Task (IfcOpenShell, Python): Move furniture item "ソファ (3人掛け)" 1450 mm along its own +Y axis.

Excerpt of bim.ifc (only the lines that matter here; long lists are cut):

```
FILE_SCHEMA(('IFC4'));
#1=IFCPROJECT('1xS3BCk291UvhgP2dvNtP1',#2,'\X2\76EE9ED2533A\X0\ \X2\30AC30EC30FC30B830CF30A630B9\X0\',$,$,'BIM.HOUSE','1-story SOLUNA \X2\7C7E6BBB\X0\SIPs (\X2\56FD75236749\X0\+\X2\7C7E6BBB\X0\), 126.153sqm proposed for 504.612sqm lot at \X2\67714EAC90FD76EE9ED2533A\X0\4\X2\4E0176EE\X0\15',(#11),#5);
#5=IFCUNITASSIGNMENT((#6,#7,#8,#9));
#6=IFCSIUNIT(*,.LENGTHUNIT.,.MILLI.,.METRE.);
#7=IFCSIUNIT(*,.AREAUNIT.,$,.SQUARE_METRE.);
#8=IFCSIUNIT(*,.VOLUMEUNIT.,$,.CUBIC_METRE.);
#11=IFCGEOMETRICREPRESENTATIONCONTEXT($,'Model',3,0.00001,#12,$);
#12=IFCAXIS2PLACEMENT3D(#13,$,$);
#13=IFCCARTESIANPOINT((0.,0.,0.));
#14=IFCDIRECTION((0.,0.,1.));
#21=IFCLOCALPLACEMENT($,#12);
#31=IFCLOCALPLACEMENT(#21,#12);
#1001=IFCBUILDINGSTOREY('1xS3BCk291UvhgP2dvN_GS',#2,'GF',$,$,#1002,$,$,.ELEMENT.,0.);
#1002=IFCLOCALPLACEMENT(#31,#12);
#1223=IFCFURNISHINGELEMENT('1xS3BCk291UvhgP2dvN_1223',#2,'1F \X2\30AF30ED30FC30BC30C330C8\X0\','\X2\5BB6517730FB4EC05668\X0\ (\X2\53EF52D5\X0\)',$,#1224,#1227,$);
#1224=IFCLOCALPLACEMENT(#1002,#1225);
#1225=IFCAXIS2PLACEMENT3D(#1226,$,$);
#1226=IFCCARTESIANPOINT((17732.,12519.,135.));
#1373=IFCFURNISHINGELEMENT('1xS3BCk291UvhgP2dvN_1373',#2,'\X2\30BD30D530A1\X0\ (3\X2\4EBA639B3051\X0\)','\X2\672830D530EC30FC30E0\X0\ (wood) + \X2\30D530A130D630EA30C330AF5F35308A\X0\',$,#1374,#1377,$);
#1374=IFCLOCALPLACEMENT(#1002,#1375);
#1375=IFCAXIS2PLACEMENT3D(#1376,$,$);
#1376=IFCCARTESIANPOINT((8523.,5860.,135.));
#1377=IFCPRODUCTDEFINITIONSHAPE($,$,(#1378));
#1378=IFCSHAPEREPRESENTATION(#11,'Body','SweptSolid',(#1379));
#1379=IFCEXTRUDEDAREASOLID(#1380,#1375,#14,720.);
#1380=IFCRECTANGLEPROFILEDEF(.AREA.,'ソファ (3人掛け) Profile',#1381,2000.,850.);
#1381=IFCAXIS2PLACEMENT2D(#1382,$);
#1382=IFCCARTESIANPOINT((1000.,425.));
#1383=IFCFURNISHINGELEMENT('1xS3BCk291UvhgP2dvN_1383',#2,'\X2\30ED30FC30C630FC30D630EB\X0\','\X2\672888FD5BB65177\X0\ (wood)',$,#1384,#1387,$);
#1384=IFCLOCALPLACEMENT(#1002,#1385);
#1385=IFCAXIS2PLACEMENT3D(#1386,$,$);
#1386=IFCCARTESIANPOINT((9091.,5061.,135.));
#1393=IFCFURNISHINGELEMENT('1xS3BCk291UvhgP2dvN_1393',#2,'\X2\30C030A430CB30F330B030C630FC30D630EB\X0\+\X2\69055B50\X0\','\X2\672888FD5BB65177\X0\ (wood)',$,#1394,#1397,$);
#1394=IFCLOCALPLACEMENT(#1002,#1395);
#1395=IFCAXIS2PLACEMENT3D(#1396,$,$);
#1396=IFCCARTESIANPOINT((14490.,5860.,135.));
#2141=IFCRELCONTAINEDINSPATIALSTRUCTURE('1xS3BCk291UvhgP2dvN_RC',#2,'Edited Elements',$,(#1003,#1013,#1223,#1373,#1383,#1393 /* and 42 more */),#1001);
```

```python
import ifcopenshell
import ifcopenshell.api.geometry
import ifcopenshell.util.placement
import ifcopenshell.util.unit

model = ifcopenshell.open("bim.ifc")
unit_scale = ifcopenshell.util.unit.calculate_unit_scale(model)

item = model.by_guid("1xS3BCk291UvhgP2dvN_1373")
matrix = ifcopenshell.util.placement.get_local_placement(item.ObjectPlacement)
matrix[:3, 3] += matrix[:3, 1] * 1.45 / unit_scale
ifcopenshell.api.geometry.edit_object_placement(model, product=item, matrix=matrix, is_si=False)

print(ifcopenshell.util.placement.get_local_placement(item.ObjectPlacement).round(3) + 0.0)

model.write("bim-out.ifc")
```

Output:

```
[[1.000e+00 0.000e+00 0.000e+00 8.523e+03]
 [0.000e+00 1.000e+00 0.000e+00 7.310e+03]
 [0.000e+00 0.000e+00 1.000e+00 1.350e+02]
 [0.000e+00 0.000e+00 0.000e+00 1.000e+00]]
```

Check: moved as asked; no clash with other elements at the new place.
